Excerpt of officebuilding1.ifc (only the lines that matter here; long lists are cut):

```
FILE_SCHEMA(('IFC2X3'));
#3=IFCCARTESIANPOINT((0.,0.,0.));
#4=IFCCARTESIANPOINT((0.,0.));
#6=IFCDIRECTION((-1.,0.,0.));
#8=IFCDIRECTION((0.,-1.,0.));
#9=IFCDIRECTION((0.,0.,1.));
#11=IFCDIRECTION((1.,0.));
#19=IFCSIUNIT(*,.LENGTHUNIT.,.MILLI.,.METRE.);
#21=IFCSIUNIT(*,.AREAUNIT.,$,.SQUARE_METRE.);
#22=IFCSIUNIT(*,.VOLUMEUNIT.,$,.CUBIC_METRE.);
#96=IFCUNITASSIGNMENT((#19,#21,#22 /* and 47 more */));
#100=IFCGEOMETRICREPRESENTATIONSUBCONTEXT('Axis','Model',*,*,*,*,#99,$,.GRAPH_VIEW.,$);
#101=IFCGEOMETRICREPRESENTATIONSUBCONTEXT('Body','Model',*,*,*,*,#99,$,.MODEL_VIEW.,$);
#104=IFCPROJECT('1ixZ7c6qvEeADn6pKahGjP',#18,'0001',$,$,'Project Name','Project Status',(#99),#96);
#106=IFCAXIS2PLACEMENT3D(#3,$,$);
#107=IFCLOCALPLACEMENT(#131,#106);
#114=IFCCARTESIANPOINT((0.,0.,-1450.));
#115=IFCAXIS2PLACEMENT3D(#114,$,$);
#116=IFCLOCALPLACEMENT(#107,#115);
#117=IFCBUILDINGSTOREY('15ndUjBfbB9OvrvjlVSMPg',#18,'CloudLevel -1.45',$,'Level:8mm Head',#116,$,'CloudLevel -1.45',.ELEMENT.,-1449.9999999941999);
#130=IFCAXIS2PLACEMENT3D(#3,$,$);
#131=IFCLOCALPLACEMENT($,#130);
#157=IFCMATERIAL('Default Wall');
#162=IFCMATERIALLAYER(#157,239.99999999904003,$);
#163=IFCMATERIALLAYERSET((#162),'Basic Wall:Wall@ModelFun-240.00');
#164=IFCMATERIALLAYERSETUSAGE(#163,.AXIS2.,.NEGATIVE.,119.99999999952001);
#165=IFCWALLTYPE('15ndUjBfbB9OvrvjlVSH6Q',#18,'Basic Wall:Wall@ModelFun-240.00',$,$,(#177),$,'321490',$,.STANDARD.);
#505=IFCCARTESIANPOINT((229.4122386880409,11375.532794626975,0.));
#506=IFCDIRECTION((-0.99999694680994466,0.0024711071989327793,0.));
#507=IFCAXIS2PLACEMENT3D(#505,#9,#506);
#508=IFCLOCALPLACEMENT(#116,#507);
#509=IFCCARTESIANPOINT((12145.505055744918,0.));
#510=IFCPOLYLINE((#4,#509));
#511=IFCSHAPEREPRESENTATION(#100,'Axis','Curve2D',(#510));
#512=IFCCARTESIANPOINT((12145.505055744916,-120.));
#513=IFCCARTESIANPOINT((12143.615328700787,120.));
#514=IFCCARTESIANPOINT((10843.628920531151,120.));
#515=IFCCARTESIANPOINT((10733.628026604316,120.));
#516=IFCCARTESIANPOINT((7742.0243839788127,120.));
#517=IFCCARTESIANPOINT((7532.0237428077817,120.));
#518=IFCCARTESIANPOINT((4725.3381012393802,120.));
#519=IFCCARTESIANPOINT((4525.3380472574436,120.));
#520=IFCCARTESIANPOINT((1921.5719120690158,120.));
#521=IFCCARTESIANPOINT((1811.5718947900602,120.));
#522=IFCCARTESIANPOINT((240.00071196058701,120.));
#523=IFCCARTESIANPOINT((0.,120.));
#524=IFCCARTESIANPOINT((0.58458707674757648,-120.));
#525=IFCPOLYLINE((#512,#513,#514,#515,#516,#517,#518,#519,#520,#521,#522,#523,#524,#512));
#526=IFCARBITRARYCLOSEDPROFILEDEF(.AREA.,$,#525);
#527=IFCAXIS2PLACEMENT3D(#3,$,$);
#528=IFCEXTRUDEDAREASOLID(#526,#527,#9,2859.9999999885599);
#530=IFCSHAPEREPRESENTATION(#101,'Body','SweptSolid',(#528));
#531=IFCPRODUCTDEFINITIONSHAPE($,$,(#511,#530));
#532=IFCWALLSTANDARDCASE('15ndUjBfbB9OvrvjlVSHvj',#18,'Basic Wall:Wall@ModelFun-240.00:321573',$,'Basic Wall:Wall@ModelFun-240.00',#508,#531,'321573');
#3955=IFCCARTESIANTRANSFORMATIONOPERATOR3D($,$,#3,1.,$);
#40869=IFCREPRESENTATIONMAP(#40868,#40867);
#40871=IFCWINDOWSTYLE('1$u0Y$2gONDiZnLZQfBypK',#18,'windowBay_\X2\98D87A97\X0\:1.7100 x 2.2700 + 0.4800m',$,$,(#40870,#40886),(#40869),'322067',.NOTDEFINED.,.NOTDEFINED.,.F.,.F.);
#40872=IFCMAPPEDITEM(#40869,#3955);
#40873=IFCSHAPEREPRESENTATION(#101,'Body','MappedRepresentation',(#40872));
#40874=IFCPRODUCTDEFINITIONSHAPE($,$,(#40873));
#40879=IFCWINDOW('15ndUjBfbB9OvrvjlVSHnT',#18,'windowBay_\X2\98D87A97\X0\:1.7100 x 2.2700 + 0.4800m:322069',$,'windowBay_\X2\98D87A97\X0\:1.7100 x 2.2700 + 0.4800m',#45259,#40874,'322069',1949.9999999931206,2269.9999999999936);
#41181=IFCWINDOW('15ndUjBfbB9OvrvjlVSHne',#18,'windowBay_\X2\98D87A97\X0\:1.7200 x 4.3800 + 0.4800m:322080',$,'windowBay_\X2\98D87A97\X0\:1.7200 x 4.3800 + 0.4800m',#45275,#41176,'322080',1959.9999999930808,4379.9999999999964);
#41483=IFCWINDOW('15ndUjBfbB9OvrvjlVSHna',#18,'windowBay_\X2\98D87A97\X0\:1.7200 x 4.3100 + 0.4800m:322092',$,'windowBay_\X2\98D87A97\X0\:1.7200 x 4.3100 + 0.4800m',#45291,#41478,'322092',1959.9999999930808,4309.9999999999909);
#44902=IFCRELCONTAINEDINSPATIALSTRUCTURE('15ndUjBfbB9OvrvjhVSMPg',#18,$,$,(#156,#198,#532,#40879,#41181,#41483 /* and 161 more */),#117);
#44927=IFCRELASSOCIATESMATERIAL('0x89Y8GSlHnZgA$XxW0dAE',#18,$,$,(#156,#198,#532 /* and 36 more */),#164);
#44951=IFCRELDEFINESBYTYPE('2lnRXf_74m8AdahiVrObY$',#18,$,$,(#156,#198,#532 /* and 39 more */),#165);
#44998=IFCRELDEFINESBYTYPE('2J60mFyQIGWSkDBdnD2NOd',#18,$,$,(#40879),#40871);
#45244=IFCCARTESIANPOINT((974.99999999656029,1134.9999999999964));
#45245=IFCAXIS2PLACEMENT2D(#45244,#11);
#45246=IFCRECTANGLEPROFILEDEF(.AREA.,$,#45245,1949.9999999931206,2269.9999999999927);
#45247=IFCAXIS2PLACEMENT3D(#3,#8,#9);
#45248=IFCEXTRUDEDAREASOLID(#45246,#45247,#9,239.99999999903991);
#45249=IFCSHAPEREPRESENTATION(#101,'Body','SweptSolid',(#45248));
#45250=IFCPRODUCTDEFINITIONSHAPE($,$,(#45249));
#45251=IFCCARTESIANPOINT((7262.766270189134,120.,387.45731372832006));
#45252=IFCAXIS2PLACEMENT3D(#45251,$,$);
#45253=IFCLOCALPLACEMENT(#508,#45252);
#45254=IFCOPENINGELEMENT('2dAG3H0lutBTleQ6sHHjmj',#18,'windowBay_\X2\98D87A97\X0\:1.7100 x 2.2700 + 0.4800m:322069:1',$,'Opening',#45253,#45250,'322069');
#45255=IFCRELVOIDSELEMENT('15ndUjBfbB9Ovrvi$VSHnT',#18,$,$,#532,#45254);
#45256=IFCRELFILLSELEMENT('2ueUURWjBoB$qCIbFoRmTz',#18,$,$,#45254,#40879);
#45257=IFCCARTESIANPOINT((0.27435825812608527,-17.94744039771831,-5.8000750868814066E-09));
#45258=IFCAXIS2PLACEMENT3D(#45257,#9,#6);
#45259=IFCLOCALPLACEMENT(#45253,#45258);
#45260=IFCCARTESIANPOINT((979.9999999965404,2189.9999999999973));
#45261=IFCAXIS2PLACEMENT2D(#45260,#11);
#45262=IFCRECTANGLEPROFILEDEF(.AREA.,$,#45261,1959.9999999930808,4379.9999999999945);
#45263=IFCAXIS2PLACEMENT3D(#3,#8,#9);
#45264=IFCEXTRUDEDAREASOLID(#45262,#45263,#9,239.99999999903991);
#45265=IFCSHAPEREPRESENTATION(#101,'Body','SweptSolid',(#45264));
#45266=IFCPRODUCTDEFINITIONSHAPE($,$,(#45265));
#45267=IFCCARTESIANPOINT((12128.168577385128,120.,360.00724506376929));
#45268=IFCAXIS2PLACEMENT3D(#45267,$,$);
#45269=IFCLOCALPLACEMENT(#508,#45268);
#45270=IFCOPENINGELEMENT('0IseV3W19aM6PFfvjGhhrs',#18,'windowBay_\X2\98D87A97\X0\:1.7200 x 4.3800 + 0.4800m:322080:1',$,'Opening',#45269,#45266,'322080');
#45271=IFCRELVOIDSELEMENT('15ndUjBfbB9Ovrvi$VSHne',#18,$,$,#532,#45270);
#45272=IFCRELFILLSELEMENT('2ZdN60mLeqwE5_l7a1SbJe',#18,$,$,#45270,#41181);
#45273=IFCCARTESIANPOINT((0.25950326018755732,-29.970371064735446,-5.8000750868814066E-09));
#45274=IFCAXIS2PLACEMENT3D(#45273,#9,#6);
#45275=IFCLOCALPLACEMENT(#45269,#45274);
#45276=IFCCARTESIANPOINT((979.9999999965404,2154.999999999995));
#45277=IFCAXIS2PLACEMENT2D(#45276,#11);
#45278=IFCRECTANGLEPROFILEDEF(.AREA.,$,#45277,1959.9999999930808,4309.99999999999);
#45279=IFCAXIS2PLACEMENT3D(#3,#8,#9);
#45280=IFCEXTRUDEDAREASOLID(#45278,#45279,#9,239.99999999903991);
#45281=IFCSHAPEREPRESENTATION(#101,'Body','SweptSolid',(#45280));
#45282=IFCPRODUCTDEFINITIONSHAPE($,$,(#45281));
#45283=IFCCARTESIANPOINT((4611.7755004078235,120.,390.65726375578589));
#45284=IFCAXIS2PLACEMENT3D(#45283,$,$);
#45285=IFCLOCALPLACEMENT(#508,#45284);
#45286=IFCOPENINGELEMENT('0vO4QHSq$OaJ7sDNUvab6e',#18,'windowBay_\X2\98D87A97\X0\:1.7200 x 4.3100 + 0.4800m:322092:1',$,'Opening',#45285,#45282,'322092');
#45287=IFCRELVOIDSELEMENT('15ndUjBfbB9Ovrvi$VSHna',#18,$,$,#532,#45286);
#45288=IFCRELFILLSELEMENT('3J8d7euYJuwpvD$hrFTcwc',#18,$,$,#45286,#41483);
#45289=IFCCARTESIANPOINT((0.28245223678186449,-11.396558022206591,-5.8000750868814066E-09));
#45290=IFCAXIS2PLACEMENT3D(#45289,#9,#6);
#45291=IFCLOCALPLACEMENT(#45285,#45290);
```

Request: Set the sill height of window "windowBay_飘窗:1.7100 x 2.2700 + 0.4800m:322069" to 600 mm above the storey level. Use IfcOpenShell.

```python
import numpy as np
import ifcopenshell
import ifcopenshell.api.geometry
import ifcopenshell.geom
import ifcopenshell.util.element
import ifcopenshell.util.placement
import ifcopenshell.util.shape
import ifcopenshell.util.unit

model = ifcopenshell.open("officebuilding1.ifc")
unit_scale = ifcopenshell.util.unit.calculate_unit_scale(model)

window = model.by_id(40879)
opening = window.FillsVoids[0].RelatingOpeningElement
storey = ifcopenshell.util.element.get_container(window, ifc_class="IfcBuildingStorey")
level = ifcopenshell.util.placement.get_local_placement(storey.ObjectPlacement)[2, 3]

# The opening's origin need not be at the sill, so measure its lowest point.
shape = ifcopenshell.geom.create_shape(ifcopenshell.geom.settings(), opening)
bottom = ifcopenshell.util.shape.get_shape_bottom_elevation(shape, shape.geometry) / unit_scale
dz = level + 0.6 / unit_scale - bottom

shift = np.array([0.0, 0.0, dz])
# The window is placed relative to its opening, so it follows when the opening moves.
matrix = ifcopenshell.util.placement.get_local_placement(opening.ObjectPlacement)
matrix[:3, 3] += shift
ifcopenshell.api.geometry.edit_object_placement(
    model, product=opening, matrix=matrix, is_si=False, should_transform_children=True
)

print(f"moved by {dz * unit_scale:+.3f} m")

model.write("officebuilding1_updated.ifc")
```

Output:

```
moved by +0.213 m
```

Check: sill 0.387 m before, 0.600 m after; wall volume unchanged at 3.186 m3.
